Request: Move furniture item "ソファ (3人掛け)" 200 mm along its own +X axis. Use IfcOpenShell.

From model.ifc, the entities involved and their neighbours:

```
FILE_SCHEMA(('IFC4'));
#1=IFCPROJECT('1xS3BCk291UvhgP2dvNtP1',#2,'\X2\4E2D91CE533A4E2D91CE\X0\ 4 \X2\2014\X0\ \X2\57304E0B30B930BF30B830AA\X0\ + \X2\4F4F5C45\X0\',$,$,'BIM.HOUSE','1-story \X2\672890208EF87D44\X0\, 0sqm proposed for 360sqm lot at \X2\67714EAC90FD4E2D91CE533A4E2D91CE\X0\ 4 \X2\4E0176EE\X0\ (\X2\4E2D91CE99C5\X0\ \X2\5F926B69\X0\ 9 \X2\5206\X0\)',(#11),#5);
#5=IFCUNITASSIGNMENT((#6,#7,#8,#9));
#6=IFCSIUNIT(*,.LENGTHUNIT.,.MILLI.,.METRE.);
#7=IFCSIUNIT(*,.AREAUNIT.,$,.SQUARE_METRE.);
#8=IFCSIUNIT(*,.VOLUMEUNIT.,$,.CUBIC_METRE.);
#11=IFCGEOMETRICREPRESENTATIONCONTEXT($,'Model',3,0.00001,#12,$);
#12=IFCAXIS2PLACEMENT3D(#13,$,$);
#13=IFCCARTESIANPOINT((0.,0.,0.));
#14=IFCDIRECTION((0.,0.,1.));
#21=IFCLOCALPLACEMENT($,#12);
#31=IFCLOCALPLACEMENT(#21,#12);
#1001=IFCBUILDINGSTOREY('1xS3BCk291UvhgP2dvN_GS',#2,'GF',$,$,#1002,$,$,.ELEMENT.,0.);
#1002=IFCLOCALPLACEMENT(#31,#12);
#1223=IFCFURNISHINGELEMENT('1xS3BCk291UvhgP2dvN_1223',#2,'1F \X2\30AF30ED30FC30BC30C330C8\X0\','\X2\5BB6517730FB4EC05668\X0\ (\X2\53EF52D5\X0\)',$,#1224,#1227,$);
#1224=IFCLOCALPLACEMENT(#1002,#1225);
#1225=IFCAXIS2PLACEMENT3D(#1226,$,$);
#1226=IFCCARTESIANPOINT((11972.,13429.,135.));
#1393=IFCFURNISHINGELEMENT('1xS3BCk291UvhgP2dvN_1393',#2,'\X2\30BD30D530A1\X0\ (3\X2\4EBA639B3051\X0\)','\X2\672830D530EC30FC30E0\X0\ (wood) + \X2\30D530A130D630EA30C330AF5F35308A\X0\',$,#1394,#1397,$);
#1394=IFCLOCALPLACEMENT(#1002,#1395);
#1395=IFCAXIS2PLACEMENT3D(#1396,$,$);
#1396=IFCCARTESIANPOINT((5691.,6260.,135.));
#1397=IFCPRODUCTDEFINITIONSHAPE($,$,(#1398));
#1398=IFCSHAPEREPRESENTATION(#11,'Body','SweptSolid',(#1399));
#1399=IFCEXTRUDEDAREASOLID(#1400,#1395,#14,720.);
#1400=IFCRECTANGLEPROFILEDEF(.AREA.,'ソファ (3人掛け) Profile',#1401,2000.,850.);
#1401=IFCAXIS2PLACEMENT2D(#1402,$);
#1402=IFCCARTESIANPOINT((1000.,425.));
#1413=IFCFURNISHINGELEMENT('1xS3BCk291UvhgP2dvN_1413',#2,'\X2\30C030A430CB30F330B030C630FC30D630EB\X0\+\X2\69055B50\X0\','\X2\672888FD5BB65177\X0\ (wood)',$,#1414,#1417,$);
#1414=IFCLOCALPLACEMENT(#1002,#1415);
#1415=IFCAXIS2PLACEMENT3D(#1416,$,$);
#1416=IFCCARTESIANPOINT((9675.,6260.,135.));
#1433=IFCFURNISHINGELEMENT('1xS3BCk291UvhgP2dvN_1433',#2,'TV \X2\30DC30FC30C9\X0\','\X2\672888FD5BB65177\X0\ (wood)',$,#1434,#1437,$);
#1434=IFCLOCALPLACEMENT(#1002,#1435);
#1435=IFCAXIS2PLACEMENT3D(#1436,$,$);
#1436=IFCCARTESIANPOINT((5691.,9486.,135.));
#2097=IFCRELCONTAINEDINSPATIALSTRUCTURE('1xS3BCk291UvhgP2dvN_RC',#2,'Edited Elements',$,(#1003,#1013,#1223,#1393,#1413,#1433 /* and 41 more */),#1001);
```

```python
import ifcopenshell
import ifcopenshell.api.geometry
import ifcopenshell.util.placement
import ifcopenshell.util.unit

model = ifcopenshell.open("model.ifc")
unit_scale = ifcopenshell.util.unit.calculate_unit_scale(model)

item = model.by_guid("1xS3BCk291UvhgP2dvN_1393")
matrix = ifcopenshell.util.placement.get_local_placement(item.ObjectPlacement)
matrix[:3, 3] += matrix[:3, 0] * 0.2 / unit_scale
ifcopenshell.api.geometry.edit_object_placement(model, product=item, matrix=matrix, is_si=False)

print(ifcopenshell.util.placement.get_local_placement(item.ObjectPlacement).round(3) + 0.0)

model.write("model_updated.ifc")
```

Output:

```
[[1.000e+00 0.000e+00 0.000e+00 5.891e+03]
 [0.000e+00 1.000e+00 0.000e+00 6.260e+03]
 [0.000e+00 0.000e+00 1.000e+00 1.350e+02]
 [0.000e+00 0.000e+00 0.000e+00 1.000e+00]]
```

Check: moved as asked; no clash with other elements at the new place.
